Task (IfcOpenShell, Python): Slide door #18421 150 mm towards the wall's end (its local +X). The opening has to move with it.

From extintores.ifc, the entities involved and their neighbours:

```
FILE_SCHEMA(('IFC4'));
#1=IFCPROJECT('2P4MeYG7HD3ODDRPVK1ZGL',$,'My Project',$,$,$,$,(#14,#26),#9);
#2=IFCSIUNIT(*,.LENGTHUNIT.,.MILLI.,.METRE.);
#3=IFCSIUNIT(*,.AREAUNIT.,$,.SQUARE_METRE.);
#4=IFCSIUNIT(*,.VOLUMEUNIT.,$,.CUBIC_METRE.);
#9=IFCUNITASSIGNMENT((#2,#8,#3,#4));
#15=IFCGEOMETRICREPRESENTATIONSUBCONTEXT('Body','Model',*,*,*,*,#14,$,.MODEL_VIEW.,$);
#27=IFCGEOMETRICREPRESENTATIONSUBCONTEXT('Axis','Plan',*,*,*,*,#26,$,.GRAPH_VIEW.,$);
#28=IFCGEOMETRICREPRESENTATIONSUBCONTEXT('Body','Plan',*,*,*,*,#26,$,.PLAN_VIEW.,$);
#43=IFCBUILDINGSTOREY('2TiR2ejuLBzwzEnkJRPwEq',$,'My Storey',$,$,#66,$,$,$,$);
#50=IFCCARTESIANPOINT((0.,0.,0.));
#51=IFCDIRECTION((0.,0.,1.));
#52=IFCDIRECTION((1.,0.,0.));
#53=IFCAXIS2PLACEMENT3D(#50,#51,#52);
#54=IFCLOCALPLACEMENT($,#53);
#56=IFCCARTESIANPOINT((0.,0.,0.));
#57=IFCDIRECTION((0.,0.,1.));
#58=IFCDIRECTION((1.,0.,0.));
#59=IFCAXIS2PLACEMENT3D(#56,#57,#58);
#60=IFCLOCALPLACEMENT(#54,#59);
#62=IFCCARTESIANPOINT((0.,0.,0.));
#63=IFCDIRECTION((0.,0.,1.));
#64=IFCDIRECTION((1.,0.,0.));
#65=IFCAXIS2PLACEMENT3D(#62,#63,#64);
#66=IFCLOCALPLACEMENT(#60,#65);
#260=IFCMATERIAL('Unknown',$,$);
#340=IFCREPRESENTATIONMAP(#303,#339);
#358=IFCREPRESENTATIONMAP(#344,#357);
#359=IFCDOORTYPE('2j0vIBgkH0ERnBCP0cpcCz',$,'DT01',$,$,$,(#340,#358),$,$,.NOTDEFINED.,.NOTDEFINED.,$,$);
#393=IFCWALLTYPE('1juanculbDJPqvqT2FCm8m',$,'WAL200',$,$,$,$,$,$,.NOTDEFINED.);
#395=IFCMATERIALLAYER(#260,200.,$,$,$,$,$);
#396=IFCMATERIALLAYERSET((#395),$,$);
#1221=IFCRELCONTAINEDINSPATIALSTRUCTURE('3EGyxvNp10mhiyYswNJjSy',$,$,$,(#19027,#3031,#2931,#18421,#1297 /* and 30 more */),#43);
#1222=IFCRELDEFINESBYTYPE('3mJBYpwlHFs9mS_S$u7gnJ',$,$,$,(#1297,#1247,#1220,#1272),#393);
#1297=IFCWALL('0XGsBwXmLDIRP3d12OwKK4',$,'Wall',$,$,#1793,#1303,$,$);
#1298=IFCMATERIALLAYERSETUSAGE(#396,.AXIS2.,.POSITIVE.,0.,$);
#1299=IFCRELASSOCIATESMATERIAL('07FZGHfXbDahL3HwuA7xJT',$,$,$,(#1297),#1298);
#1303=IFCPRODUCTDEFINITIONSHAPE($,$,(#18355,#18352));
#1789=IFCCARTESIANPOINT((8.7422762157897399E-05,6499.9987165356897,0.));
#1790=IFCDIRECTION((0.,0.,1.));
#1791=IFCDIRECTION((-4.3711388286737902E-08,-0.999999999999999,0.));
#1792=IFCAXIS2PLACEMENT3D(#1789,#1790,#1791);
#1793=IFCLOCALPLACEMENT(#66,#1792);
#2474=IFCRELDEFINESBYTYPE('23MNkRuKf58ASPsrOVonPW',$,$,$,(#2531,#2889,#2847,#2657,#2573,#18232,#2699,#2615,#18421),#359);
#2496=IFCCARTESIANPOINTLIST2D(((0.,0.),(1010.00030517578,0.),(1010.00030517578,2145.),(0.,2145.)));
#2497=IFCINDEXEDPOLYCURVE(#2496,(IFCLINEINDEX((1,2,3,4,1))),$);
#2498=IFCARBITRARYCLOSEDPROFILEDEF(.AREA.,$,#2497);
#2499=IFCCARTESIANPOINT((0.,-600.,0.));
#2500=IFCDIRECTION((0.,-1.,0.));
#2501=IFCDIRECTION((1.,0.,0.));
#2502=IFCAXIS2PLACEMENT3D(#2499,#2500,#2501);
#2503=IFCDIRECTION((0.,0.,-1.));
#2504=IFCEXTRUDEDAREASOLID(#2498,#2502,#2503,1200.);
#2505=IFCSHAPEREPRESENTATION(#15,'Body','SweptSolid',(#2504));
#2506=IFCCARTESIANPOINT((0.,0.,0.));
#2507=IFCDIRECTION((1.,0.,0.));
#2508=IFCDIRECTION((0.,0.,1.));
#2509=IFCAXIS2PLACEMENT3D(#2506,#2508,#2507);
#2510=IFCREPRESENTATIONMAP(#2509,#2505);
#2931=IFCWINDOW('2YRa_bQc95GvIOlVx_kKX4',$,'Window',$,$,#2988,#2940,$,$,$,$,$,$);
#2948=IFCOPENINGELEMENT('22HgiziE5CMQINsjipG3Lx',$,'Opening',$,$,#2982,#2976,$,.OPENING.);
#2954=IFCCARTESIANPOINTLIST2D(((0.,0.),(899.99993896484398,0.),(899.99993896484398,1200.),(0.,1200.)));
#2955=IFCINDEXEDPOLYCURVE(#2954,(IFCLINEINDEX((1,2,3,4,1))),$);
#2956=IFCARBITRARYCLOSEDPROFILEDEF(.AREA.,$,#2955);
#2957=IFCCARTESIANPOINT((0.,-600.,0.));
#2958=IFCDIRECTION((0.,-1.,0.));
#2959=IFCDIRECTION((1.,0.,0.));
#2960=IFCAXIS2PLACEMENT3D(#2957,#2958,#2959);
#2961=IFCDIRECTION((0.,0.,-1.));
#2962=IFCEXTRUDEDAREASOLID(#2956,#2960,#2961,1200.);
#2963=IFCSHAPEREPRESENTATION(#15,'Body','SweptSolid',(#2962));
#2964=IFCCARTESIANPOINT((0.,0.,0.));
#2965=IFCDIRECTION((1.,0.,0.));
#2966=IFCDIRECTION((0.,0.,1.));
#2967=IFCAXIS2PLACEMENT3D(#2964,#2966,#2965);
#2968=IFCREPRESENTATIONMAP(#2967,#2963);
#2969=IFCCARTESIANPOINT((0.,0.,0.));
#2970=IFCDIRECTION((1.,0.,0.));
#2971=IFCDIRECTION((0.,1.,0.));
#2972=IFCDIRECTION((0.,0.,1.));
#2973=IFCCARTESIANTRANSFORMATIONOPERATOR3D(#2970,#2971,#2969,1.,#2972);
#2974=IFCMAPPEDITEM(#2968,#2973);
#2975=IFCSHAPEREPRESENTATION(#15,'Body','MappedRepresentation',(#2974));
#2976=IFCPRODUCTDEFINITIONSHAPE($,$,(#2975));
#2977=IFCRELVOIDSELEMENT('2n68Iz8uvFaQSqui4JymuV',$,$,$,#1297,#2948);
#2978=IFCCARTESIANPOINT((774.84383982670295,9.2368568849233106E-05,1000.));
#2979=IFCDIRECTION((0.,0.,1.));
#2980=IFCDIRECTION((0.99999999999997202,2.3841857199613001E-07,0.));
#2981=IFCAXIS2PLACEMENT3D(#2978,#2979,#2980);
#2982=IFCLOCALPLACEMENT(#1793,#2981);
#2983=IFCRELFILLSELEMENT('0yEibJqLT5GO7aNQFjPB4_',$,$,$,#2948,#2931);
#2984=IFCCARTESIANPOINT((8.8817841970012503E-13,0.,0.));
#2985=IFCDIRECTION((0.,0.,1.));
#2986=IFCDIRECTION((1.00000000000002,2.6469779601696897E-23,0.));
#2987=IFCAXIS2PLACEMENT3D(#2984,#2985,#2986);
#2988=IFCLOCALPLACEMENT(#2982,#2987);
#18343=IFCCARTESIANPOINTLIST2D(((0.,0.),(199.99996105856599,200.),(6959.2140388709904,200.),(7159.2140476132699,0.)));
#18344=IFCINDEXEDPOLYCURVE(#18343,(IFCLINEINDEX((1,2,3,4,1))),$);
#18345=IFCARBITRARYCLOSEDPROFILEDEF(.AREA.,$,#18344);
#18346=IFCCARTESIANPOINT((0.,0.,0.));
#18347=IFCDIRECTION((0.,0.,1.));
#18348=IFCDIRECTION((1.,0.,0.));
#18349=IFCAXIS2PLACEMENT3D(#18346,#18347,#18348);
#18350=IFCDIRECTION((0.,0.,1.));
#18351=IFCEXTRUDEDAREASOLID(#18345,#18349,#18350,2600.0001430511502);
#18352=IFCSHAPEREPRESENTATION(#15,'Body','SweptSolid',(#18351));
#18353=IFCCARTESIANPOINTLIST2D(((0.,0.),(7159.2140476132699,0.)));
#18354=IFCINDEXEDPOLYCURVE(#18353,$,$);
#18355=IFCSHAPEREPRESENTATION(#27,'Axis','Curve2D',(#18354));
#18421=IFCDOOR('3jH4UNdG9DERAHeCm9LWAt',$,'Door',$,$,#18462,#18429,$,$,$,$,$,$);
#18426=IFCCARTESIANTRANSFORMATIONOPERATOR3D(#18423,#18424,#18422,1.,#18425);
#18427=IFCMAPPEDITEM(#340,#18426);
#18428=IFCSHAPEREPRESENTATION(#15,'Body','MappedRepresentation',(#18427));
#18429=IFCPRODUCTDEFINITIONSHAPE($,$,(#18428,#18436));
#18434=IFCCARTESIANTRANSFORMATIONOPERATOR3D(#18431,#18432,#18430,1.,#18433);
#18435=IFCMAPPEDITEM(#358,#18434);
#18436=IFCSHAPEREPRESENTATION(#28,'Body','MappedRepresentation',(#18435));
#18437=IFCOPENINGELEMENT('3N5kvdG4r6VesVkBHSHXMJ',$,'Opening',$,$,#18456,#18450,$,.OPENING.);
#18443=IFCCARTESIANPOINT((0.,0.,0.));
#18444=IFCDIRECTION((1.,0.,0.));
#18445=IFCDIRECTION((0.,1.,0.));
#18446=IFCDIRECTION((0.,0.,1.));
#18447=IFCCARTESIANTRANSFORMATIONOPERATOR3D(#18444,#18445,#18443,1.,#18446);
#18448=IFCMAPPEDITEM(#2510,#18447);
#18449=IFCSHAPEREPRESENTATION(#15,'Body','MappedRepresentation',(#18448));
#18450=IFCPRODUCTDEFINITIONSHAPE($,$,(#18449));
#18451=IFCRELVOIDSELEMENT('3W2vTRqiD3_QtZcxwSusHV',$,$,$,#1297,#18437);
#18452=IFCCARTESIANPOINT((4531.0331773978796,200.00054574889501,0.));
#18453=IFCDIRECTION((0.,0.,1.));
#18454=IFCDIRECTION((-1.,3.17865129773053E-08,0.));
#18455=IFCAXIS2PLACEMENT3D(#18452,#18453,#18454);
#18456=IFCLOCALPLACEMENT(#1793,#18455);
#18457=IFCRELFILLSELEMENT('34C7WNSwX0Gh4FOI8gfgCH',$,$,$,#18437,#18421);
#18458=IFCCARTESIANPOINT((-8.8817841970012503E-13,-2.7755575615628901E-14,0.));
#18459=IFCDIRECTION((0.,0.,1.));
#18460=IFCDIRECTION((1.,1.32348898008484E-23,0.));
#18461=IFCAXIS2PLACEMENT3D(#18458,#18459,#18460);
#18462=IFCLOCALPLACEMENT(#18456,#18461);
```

```python
import ifcopenshell
import ifcopenshell.api.geometry
import ifcopenshell.util.placement
import ifcopenshell.util.unit

model = ifcopenshell.open("extintores.ifc")
unit_scale = ifcopenshell.util.unit.calculate_unit_scale(model)

door = model.by_guid("3jH4UNdG9DERAHeCm9LWAt")
opening = door.FillsVoids[0].RelatingOpeningElement
wall = opening.VoidsElements[0].RelatingBuildingElement

wall_matrix = ifcopenshell.util.placement.get_local_placement(wall.ObjectPlacement)
shift = wall_matrix[:3, 0] * 0.15 / unit_scale
before = ifcopenshell.util.placement.get_local_placement(door.ObjectPlacement)[:3, 3].copy()

# The door is placed relative to its opening, so it follows when the opening moves.
matrix = ifcopenshell.util.placement.get_local_placement(opening.ObjectPlacement)
matrix[:3, 3] += shift
ifcopenshell.api.geometry.edit_object_placement(
    model, product=opening, matrix=matrix, is_si=False, should_transform_children=True
)

after = ifcopenshell.util.placement.get_local_placement(door.ObjectPlacement)[:3, 3]
print("door moved by", (after - before).round(3) + 0.0)

model.write("extintores_edited.ifc")
```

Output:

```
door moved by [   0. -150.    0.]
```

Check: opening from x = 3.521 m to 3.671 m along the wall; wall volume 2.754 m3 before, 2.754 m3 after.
